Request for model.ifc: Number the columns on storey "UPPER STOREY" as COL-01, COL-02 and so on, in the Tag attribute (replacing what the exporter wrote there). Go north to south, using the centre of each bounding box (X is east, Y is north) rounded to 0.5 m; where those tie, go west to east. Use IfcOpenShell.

First a look at what the model holds.

```python
import ifcopenshell
import ifcopenshell.util.element
import ifcopenshell.util.placement

model = ifcopenshell.open("model.ifc")
print(model.schema)
storey = next(s for s in model.by_type("IfcBuildingStorey") if s.Name == "UPPER STOREY")
columns = [e for e in ifcopenshell.util.element.get_decomposition(storey) if e.is_a("IfcColumn")]
for e in sorted(columns, key=lambda e: e.id()):
    origin = ifcopenshell.util.placement.get_local_placement(e.ObjectPlacement)[:3, 3]
    print(e.id(), e.Tag, e.Name, origin.round(2) + 0.0, sep=" | ")
```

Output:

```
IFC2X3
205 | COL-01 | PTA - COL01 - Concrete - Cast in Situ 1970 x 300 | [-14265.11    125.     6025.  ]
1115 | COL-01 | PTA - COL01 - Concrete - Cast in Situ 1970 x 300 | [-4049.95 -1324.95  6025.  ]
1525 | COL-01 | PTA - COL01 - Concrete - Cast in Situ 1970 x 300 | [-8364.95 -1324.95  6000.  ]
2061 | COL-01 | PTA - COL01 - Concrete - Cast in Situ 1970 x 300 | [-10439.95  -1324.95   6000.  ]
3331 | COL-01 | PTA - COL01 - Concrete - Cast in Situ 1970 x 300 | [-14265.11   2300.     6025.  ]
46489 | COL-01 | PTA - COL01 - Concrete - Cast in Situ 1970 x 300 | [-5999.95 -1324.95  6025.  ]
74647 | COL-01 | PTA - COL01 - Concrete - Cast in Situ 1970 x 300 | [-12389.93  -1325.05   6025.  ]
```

```python
import ifcopenshell
import ifcopenshell.geom
import ifcopenshell.util.element
import ifcopenshell.util.shape

model = ifcopenshell.open("model.ifc")
settings = ifcopenshell.geom.settings()
settings.set("use-world-coords", True)


def centre(element):
    shape = ifcopenshell.geom.create_shape(settings, element)
    return ifcopenshell.util.shape.get_bbox_centroid(shape.geometry)


storey = next(s for s in model.by_type("IfcBuildingStorey") if s.Name == "UPPER STOREY")
columns = [e for e in ifcopenshell.util.element.get_decomposition(storey) if e.is_a("IfcColumn")]

# Insertion points can sit at a corner or the storey origin, so sort by the geometry (in metres).
centres = {e: centre(e) for e in columns}
columns.sort(key=lambda e: (-round(centres[e][1] / 0.5), centres[e][0]))

for i, e in enumerate(columns, start=1):
    number = f"COL-{i:02d}"
    e.Tag = number
    print(e.id(), number)

model.write("model_updated.ifc")
```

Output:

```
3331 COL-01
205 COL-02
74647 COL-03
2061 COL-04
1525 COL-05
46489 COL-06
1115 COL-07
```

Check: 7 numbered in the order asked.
